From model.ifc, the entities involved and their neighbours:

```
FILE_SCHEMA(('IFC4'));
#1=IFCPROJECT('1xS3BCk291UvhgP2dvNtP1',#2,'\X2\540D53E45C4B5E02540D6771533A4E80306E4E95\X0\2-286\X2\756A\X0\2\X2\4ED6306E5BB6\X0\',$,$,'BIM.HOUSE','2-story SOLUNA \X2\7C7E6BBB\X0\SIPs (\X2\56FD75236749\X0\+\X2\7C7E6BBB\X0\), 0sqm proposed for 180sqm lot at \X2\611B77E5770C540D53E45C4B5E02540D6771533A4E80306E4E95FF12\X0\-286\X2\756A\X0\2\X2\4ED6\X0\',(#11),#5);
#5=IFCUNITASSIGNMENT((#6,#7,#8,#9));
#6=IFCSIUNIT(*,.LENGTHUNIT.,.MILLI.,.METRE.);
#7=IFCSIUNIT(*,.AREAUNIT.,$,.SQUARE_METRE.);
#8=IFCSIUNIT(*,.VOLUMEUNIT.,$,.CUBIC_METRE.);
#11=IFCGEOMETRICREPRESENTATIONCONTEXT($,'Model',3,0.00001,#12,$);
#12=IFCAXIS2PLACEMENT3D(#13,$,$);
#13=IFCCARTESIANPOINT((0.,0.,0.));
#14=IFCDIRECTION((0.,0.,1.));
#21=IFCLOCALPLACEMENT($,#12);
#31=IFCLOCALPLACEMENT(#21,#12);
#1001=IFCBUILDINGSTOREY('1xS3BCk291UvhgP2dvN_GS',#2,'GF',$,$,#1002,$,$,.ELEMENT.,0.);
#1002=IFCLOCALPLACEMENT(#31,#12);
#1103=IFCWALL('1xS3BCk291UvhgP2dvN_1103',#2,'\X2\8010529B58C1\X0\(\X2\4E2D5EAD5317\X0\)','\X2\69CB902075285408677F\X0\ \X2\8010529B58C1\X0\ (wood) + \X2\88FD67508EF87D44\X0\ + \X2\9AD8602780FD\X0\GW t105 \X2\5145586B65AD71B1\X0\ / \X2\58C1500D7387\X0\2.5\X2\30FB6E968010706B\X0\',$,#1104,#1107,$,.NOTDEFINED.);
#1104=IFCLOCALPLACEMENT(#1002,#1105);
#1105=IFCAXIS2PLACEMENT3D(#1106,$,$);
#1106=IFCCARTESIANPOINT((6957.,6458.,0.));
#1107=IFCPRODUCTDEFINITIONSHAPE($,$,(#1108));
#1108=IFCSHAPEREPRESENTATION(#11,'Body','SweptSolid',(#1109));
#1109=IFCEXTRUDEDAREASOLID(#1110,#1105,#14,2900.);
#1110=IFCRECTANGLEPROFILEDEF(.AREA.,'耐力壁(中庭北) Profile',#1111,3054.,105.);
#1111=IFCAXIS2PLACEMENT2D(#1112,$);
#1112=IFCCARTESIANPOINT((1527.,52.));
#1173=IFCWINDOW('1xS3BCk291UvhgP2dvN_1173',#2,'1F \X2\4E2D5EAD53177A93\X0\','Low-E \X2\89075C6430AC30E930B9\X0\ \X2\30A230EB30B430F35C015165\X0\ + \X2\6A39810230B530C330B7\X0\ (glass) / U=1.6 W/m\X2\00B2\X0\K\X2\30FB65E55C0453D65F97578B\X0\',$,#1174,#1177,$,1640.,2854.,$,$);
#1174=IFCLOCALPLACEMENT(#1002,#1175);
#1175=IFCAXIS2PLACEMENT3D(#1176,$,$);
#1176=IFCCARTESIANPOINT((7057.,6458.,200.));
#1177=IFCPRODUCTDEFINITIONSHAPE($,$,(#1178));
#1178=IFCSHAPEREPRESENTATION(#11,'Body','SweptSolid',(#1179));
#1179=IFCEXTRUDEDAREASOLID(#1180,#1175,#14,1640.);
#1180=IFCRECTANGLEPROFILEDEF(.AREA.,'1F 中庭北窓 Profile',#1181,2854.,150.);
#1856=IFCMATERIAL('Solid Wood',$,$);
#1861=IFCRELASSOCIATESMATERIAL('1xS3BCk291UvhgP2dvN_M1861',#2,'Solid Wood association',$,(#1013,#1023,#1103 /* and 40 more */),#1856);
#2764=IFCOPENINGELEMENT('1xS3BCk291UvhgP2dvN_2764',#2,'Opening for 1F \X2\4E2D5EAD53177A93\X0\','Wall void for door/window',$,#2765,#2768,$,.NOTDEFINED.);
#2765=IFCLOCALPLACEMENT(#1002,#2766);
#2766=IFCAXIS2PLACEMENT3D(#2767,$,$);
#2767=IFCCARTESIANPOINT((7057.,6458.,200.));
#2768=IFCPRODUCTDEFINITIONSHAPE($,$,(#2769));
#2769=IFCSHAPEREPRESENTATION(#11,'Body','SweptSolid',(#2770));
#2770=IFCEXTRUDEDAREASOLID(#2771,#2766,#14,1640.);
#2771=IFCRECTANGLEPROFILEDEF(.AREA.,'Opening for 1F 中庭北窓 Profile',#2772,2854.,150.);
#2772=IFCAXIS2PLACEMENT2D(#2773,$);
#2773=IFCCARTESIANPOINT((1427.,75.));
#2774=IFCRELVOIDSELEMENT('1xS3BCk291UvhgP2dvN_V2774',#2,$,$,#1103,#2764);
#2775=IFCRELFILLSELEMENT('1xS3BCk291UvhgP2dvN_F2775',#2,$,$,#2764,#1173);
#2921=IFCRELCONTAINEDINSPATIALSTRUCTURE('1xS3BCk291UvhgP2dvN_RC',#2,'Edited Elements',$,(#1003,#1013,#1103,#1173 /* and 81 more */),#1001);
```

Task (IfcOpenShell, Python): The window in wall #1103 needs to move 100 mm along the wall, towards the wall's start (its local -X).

```python
import ifcopenshell
import ifcopenshell.api.geometry
import ifcopenshell.util.placement

model = ifcopenshell.open("model.ifc")

window = model.by_id(1173)
opening = window.FillsVoids[0].RelatingOpeningElement
wall = opening.VoidsElements[0].RelatingBuildingElement

wall_matrix = ifcopenshell.util.placement.get_local_placement(wall.ObjectPlacement)
shift = wall_matrix[:3, 0] * -100.0
before = ifcopenshell.util.placement.get_local_placement(window.ObjectPlacement)[:3, 3].copy()

# The window is not placed relative to its opening, so move both.
for product in (opening, window):
    matrix = ifcopenshell.util.placement.get_local_placement(product.ObjectPlacement)
    matrix[:3, 3] += shift
    ifcopenshell.api.geometry.edit_object_placement(model, product=product, matrix=matrix, is_si=False)

after = ifcopenshell.util.placement.get_local_placement(window.ObjectPlacement)[:3, 3]
print("window moved by", (after - before).round(3) + 0.0)

model.write("model_edited.ifc")
```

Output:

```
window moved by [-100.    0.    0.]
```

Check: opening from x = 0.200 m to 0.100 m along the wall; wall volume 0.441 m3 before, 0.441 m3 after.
